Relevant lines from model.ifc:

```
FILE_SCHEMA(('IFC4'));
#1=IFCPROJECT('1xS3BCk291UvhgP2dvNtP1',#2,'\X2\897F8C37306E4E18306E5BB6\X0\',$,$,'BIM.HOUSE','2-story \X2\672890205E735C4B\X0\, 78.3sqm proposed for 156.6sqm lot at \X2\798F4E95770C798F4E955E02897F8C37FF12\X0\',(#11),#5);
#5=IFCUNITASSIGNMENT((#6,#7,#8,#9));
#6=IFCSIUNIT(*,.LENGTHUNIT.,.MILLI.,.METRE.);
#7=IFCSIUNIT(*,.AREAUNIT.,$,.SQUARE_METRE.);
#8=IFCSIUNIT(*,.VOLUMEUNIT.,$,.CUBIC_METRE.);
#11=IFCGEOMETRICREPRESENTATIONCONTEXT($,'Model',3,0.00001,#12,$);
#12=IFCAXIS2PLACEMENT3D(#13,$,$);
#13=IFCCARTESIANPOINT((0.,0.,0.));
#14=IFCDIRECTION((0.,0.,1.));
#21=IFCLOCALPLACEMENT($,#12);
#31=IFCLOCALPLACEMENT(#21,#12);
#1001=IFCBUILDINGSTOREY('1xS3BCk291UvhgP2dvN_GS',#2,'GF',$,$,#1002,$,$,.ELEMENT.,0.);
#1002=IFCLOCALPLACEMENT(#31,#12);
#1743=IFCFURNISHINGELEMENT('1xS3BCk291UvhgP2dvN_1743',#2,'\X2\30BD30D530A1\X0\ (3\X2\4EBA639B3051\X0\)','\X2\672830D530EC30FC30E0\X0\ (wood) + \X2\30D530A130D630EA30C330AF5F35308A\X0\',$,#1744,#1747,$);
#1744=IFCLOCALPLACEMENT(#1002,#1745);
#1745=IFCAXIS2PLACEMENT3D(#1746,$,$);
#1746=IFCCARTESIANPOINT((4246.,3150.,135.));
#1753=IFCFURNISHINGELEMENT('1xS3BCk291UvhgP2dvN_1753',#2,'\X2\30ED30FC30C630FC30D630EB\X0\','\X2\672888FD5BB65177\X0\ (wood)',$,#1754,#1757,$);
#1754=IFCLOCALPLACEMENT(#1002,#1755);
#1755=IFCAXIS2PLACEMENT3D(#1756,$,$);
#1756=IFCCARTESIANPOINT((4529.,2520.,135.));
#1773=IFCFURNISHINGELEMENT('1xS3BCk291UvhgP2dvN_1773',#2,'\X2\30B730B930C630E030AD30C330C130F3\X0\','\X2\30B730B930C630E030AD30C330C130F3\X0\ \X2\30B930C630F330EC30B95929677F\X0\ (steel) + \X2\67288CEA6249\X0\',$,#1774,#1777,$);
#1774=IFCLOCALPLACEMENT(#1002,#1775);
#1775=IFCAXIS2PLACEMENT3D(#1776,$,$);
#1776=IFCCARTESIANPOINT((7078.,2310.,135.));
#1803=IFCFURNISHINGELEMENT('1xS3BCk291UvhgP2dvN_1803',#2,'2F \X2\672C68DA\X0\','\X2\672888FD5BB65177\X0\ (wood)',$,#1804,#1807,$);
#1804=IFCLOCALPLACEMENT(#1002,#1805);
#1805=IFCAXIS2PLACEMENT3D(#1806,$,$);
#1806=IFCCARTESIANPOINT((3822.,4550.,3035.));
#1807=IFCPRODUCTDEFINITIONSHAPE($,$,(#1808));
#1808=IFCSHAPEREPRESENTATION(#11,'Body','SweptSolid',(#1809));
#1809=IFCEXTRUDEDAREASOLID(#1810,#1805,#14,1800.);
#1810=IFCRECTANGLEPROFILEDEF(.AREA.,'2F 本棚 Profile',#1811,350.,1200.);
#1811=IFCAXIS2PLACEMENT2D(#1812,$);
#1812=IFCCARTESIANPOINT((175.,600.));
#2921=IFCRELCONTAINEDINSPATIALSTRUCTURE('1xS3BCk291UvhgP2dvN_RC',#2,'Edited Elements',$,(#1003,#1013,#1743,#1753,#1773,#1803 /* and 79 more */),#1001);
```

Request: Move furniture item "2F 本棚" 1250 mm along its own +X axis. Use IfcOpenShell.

```python
import ifcopenshell
import ifcopenshell.api.geometry
import ifcopenshell.util.placement

model = ifcopenshell.open("model.ifc")

item = model.by_guid("1xS3BCk291UvhgP2dvN_1803")
matrix = ifcopenshell.util.placement.get_local_placement(item.ObjectPlacement)
matrix[:3, 3] += matrix[:3, 0] * 1250.0
ifcopenshell.api.geometry.edit_object_placement(model, product=item, matrix=matrix, is_si=False)

print(ifcopenshell.util.placement.get_local_placement(item.ObjectPlacement).round(3) + 0.0)

model.write("model_edited.ifc")
```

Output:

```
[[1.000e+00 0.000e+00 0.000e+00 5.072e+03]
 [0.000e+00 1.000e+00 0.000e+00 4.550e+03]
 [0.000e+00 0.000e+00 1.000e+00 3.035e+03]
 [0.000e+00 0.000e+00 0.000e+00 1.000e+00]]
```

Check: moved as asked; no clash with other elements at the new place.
